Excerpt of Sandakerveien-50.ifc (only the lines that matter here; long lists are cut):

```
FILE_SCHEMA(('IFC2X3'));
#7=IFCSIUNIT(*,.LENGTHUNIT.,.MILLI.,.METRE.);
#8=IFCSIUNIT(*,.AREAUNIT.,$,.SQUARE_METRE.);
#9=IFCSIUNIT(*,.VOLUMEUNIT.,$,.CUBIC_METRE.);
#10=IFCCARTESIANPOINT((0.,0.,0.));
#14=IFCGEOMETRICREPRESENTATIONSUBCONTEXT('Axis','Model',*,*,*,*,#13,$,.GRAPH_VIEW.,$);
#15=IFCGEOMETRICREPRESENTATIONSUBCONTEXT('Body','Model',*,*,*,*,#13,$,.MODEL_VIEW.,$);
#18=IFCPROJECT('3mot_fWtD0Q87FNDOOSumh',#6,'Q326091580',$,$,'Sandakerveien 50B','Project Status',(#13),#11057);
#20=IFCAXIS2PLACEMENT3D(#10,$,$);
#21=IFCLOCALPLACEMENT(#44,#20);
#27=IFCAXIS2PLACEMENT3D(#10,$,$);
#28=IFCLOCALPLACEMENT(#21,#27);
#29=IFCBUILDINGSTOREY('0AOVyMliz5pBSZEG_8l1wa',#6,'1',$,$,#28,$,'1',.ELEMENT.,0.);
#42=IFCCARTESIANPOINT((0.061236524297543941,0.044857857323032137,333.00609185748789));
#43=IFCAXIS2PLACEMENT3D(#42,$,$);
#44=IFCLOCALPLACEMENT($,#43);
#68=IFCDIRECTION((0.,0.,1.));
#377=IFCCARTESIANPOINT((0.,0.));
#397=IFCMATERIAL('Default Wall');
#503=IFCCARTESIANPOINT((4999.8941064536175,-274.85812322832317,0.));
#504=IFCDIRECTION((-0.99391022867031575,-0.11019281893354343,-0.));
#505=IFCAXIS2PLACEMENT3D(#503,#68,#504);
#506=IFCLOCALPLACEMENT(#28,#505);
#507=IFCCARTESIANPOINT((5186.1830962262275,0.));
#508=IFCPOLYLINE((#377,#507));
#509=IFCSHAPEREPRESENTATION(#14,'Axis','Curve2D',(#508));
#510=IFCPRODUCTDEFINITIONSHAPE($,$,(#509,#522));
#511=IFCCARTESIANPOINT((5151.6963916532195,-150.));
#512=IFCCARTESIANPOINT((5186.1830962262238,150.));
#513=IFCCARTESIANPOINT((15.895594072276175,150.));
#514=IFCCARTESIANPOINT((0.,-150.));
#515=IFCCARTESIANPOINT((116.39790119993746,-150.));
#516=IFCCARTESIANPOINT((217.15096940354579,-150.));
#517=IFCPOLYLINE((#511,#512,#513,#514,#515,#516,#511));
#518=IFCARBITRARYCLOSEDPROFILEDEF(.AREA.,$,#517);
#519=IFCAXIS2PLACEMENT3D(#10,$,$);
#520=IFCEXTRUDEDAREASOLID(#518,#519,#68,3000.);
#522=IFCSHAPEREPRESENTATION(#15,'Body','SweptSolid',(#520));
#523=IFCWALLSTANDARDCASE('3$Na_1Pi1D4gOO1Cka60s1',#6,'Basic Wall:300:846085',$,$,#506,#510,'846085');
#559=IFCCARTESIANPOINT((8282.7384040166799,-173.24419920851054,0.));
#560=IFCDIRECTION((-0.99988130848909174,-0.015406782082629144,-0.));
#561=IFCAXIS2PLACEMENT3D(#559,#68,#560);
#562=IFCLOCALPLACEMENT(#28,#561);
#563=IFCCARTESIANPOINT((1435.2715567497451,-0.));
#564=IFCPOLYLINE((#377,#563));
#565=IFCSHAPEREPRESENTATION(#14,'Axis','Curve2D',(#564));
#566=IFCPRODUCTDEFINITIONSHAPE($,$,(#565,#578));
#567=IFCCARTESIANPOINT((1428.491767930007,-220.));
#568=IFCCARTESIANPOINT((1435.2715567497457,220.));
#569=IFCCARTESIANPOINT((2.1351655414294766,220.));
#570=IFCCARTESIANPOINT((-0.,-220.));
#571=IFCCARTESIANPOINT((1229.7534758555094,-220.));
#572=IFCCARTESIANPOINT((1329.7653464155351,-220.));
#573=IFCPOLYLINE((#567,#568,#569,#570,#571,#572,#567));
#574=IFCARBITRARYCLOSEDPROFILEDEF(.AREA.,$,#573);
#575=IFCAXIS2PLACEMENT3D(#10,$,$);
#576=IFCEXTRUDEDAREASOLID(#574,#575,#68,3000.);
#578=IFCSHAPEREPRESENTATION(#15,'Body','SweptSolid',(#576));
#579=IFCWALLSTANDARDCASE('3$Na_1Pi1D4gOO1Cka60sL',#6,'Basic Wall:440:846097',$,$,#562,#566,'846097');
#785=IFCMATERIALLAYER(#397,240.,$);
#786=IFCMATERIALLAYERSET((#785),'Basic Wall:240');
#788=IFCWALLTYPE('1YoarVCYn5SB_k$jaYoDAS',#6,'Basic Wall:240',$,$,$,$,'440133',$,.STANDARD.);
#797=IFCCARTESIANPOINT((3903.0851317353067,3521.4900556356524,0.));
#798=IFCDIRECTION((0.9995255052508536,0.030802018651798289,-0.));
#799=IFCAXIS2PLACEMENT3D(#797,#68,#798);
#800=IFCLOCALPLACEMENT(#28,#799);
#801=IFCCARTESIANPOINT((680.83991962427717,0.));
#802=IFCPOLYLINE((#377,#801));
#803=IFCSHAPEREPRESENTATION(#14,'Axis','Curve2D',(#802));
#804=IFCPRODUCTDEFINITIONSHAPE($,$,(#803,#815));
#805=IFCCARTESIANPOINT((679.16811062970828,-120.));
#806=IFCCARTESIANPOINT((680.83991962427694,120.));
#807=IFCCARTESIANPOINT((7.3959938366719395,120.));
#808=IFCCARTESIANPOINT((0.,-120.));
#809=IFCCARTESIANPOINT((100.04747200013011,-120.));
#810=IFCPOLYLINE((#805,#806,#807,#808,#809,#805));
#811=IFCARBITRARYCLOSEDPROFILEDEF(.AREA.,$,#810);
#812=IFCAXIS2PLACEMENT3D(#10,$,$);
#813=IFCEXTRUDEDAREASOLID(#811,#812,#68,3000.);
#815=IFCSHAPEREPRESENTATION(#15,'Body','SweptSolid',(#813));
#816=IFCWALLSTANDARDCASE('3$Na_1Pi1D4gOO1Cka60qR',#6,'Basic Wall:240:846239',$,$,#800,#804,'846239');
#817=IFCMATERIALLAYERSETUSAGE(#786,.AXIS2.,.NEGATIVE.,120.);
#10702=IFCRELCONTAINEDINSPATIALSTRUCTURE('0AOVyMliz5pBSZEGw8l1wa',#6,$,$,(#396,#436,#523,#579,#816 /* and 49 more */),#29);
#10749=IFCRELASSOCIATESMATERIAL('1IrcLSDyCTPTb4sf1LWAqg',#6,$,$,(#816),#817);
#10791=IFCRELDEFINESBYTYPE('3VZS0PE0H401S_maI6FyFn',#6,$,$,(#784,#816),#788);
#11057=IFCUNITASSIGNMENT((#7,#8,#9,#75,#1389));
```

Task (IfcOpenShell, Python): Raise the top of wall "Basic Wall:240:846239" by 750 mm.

```python
import ifcopenshell
import ifcopenshell.geom
import ifcopenshell.util.representation
import ifcopenshell.util.shape
import ifcopenshell.util.unit

model = ifcopenshell.open("Sandakerveien-50.ifc")
unit_scale = ifcopenshell.util.unit.calculate_unit_scale(model)
settings = ifcopenshell.geom.settings()


def volume(element):
    """Net volume in cubic metres, openings subtracted."""
    shape = ifcopenshell.geom.create_shape(settings, element)
    return ifcopenshell.util.shape.get_volume(shape.geometry)


wall = model.by_guid("3$Na_1Pi1D4gOO1Cka60qR")
before = volume(wall)

body = ifcopenshell.util.representation.get_representation(wall, "Model", "Body")
solid = body.Items[0]
old_height = solid.Depth
solid.Depth += 0.75 / unit_scale
after = volume(wall)

print(f"height {old_height:g} -> {solid.Depth:g}, volume {before:.3f} -> {after:.3f} m3")

model.write("Sandakerveien-50-out.ifc")
```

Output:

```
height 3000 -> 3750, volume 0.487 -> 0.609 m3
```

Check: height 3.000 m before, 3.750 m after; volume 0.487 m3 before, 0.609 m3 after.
